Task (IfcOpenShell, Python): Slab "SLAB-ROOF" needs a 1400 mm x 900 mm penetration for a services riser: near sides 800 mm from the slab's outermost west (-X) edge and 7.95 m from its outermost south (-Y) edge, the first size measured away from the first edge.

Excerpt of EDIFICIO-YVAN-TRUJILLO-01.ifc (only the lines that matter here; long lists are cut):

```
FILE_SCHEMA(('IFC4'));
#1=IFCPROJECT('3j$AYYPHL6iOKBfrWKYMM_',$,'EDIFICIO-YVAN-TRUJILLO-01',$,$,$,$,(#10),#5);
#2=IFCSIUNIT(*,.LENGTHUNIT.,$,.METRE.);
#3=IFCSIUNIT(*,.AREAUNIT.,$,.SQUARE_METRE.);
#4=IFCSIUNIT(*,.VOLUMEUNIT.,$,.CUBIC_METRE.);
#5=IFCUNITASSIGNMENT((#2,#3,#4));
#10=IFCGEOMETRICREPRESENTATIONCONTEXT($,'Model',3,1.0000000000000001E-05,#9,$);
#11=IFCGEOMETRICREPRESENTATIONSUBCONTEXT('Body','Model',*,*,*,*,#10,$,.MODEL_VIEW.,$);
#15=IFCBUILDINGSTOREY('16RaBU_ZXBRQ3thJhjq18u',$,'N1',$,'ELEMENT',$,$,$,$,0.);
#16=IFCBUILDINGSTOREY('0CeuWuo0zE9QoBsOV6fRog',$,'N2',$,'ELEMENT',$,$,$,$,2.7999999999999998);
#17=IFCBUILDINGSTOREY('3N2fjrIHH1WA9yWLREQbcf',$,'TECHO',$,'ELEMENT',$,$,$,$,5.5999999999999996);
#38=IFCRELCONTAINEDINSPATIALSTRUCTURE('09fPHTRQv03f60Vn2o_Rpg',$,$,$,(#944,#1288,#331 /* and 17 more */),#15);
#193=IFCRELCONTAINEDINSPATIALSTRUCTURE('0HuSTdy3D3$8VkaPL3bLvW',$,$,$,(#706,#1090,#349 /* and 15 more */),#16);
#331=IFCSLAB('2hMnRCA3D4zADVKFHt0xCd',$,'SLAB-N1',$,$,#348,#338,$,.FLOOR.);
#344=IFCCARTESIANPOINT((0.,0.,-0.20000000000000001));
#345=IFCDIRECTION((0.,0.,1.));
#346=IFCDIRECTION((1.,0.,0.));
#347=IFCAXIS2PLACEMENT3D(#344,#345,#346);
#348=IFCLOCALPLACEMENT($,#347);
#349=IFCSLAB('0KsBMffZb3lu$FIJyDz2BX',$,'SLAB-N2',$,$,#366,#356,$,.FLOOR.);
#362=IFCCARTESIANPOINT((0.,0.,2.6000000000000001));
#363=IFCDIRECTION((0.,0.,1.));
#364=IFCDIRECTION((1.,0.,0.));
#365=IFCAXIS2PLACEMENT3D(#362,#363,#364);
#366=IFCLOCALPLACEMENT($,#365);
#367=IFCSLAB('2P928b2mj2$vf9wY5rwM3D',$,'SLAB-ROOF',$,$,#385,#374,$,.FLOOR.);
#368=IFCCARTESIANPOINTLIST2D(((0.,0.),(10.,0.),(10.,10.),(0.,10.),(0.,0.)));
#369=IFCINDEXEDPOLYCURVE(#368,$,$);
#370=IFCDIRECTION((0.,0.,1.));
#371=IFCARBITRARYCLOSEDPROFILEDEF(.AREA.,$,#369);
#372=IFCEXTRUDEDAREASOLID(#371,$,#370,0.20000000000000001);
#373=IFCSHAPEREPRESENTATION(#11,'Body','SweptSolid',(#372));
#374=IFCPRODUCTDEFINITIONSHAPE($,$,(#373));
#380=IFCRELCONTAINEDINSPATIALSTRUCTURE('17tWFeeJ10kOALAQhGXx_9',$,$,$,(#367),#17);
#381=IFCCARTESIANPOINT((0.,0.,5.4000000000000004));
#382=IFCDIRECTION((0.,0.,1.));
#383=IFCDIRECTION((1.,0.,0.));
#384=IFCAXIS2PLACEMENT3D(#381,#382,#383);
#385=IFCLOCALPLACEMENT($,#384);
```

```python
import numpy as np
import ifcopenshell
import ifcopenshell.api.feature
import ifcopenshell.api.geometry
import ifcopenshell.api.root
import ifcopenshell.geom
import ifcopenshell.util.placement
import ifcopenshell.util.representation
import ifcopenshell.util.shape
import ifcopenshell.util.unit

model = ifcopenshell.open("EDIFICIO-YVAN-TRUJILLO-01.ifc")
unit_scale = ifcopenshell.util.unit.calculate_unit_scale(model)
settings = ifcopenshell.geom.settings()


def volume(element):
    """Net volume in cubic metres, openings subtracted."""
    shape = ifcopenshell.geom.create_shape(settings, element)
    return ifcopenshell.util.shape.get_volume(shape.geometry)


slab = model.by_id(367)
before = volume(slab)

# Extent in the slab's own axes, in metres. The edges named are its -X and -Y sides.
slab_shape = ifcopenshell.geom.create_shape(settings, slab)
vertices = ifcopenshell.util.shape.get_vertices(slab_shape.geometry)
x_min, y_min, bottom = vertices.min(axis=0)
top = vertices[:, 2].max()

opening = ifcopenshell.api.root.create_entity(model, ifc_class="IfcOpeningElement", name="Services riser opening", predefined_type="OPENING")
context = ifcopenshell.util.representation.get_context(model, "Model", "Body", "MODEL_VIEW")
width, depth = 1.4, 0.9
outline = [(0.0, 0.0), (width, 0.0), (width, depth), (0.0, depth), (0.0, 0.0)]
# Overshoot both faces by 50 mm so the cut is clean.
shape = ifcopenshell.api.geometry.add_slab_representation(
    model, context=context, depth=top - bottom + 0.1, polyline=outline
)
ifcopenshell.api.geometry.assign_representation(model, product=opening, representation=shape)

matrix = ifcopenshell.util.placement.get_local_placement(slab.ObjectPlacement)
matrix[:, 3] = matrix @ np.append(np.array([x_min + 0.8, y_min + 7.95, bottom - 0.05]) / unit_scale, 1.0)
ifcopenshell.api.geometry.edit_object_placement(model, product=opening, matrix=matrix, is_si=False)
ifcopenshell.api.feature.add_feature(model, feature=opening, element=slab)

after = volume(slab)

print(f"slab volume {before:.3f} -> {after:.3f} m3")

model.write("EDIFICIO-YVAN-TRUJILLO-01_updated.ifc")
```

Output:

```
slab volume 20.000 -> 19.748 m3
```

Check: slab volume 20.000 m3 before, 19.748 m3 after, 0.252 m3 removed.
